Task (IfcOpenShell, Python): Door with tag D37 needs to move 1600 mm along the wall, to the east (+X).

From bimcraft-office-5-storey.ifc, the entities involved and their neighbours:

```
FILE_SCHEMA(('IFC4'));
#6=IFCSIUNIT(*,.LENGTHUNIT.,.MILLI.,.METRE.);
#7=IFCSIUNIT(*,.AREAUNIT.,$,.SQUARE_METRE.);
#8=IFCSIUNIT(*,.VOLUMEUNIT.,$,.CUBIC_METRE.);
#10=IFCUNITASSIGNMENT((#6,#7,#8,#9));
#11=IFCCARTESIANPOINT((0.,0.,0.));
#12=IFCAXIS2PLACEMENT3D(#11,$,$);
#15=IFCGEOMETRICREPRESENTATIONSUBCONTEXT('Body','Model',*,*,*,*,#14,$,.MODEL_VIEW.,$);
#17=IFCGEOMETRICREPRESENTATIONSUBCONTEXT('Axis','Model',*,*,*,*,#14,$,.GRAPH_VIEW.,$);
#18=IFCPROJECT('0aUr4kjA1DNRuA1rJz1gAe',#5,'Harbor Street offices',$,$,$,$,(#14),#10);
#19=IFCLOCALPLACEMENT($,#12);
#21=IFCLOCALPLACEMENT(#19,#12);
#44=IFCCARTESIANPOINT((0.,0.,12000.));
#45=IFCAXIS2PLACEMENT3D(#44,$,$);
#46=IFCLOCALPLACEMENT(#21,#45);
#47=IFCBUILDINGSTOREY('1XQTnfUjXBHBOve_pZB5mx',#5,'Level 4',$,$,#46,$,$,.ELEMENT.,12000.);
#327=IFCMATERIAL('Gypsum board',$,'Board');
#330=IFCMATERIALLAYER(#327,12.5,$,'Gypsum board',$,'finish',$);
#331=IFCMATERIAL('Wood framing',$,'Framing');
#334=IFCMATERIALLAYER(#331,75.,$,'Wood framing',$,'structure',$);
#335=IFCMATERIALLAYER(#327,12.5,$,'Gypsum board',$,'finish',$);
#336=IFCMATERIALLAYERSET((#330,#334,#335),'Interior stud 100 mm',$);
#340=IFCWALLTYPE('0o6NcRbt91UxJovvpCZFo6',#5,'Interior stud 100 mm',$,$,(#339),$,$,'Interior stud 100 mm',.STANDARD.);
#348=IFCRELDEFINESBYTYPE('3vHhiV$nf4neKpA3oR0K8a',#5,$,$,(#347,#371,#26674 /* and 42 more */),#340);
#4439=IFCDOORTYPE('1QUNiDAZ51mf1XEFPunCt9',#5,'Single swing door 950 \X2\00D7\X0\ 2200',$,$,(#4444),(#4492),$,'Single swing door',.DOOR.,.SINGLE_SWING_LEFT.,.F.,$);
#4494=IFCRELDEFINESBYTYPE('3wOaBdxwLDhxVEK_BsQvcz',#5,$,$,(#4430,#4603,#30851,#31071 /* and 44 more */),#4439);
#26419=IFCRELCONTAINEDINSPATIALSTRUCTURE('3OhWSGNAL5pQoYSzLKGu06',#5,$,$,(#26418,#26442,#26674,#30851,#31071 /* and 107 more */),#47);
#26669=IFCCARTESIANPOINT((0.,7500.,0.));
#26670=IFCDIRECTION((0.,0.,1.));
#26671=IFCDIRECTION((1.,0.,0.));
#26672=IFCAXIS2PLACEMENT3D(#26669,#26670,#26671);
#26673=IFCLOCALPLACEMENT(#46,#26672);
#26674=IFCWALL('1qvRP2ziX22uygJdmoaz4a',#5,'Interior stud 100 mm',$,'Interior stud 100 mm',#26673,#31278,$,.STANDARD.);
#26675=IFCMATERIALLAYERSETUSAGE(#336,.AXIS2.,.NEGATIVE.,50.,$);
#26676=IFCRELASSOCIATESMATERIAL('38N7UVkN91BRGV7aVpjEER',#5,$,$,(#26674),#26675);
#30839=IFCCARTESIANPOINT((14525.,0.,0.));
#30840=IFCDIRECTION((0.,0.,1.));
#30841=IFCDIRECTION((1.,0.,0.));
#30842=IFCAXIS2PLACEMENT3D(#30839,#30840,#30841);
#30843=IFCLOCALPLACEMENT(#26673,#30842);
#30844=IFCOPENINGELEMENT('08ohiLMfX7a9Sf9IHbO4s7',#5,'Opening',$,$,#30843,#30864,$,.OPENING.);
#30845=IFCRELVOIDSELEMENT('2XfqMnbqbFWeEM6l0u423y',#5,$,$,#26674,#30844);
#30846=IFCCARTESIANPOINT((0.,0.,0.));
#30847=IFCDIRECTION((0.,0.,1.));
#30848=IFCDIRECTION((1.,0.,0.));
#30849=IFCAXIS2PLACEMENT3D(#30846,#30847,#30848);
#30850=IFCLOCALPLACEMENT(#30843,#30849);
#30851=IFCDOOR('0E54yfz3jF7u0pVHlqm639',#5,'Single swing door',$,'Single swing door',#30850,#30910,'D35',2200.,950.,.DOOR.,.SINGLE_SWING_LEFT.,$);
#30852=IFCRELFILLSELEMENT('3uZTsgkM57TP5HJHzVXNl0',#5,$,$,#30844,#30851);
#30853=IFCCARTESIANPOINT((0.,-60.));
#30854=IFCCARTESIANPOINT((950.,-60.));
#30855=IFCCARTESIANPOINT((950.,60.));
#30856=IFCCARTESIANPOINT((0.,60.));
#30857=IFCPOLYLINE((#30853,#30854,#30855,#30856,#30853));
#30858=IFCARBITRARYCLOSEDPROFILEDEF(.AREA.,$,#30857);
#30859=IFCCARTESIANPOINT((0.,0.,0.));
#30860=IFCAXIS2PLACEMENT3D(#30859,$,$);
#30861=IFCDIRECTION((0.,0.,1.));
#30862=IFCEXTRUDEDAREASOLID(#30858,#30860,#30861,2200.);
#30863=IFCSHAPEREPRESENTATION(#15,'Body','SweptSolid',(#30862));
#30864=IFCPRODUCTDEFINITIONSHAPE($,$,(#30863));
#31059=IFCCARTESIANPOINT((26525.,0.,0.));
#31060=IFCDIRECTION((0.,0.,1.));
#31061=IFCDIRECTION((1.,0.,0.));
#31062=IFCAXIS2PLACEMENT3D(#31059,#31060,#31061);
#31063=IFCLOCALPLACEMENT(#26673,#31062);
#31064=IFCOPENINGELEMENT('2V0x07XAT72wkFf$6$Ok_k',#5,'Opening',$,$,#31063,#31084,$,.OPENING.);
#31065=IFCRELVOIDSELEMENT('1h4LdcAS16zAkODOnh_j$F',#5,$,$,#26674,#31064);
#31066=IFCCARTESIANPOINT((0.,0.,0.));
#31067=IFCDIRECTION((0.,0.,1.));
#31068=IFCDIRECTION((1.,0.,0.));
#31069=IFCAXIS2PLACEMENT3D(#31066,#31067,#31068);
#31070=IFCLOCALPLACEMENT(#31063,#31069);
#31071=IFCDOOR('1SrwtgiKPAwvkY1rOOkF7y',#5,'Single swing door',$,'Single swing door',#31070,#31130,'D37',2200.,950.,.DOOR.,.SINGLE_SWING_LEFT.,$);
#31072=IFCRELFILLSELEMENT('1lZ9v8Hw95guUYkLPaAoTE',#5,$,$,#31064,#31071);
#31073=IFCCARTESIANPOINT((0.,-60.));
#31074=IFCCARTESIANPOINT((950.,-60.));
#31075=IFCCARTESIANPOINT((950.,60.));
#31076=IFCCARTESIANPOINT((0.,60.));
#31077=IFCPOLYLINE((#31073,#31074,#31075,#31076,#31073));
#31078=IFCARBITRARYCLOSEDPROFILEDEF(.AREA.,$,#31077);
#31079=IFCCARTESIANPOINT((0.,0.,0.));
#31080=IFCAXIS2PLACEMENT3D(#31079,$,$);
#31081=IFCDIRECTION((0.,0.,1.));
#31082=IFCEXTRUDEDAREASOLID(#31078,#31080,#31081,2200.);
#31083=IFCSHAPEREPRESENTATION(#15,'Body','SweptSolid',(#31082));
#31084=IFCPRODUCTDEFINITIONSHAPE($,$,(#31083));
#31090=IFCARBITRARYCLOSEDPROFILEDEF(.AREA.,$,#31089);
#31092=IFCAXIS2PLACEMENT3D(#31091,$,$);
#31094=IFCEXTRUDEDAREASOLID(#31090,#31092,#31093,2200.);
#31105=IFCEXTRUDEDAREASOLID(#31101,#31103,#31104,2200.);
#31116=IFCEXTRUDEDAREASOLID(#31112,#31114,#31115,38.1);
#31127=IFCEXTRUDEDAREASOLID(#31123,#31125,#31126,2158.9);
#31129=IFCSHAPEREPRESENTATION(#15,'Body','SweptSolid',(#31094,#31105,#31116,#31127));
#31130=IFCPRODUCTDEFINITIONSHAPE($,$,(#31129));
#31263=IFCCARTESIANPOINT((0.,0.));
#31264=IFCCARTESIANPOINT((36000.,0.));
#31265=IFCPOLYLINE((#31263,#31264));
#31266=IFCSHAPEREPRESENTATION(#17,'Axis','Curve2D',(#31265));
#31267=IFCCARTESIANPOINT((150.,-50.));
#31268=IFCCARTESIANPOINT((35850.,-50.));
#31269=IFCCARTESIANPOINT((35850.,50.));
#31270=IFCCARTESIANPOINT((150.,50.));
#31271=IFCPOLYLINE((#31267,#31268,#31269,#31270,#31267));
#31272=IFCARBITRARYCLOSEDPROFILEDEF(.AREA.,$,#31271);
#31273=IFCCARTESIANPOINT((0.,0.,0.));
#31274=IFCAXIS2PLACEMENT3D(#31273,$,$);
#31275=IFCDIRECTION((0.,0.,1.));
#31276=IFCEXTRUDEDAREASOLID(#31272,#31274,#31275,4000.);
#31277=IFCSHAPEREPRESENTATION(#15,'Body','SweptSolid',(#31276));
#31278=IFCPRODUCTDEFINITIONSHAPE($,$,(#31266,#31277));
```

```python
import ifcopenshell
import ifcopenshell.api.geometry
import ifcopenshell.util.placement

model = ifcopenshell.open("bimcraft-office-5-storey.ifc")

door = model.by_id(31071)
opening = door.FillsVoids[0].RelatingOpeningElement
wall = opening.VoidsElements[0].RelatingBuildingElement

wall_matrix = ifcopenshell.util.placement.get_local_placement(wall.ObjectPlacement)
shift = wall_matrix[:3, 0] * 1600.0
before = ifcopenshell.util.placement.get_local_placement(door.ObjectPlacement)[:3, 3].copy()

# The door is placed relative to its opening, so it follows when the opening moves.
matrix = ifcopenshell.util.placement.get_local_placement(opening.ObjectPlacement)
matrix[:3, 3] += shift
ifcopenshell.api.geometry.edit_object_placement(
    model, product=opening, matrix=matrix, is_si=False, should_transform_children=True
)

after = ifcopenshell.util.placement.get_local_placement(door.ObjectPlacement)[:3, 3]
print("door moved by", (after - before).round(3) + 0.0)

model.write("bimcraft-office-5-storey_updated.ifc")
```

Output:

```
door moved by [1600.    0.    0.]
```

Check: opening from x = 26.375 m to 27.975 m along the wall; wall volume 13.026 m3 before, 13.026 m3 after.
